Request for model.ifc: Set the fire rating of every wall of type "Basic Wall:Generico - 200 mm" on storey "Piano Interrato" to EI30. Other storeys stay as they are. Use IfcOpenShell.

First a look at what the model holds.

```python
import ifcopenshell
import ifcopenshell.util.element

model = ifcopenshell.open("model.ifc")
print(model.schema)
storey = next(s for s in model.by_type("IfcBuildingStorey") if s.Name == "Piano Interrato")
walls = [e for e in ifcopenshell.util.element.get_decomposition(storey) if e.is_a("IfcWall")]
seen = {}
for e in walls:
    element_type = ifcopenshell.util.element.get_type(e)
    key = (element_type.Name if element_type != e and element_type else None, ifcopenshell.util.element.get_pset(e, "Pset_WallCommon", "FireRating"))
    seen[key] = seen.get(key, 0) + 1
for (name, value), count in sorted(seen.items(), key=str):
    print(count, "x", name, "|", value)
```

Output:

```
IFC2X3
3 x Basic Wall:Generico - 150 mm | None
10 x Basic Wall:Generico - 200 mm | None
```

```python
import ifcopenshell
import ifcopenshell.api.pset
import ifcopenshell.util.element

model = ifcopenshell.open("model.ifc")

storey = next(s for s in model.by_type("IfcBuildingStorey") if s.Name == "Piano Interrato")
walls = [e for e in ifcopenshell.util.element.get_decomposition(storey) if e.is_a("IfcWall")]

count = 0
for e in walls:
    element_type = ifcopenshell.util.element.get_type(e)
    if element_type in (None, e) or element_type.Name != "Basic Wall:Generico - 200 mm":
        continue
    # add_pset returns the element's existing set when there is one.
    pset = ifcopenshell.api.pset.add_pset(model, product=e, name="Pset_WallCommon")
    ifcopenshell.api.pset.edit_pset(model, pset=pset, properties={"FireRating": "EI30"})
    count += 1

print(count, "walls updated")

model.write("model_rev.ifc")
```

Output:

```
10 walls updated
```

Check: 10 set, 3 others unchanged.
